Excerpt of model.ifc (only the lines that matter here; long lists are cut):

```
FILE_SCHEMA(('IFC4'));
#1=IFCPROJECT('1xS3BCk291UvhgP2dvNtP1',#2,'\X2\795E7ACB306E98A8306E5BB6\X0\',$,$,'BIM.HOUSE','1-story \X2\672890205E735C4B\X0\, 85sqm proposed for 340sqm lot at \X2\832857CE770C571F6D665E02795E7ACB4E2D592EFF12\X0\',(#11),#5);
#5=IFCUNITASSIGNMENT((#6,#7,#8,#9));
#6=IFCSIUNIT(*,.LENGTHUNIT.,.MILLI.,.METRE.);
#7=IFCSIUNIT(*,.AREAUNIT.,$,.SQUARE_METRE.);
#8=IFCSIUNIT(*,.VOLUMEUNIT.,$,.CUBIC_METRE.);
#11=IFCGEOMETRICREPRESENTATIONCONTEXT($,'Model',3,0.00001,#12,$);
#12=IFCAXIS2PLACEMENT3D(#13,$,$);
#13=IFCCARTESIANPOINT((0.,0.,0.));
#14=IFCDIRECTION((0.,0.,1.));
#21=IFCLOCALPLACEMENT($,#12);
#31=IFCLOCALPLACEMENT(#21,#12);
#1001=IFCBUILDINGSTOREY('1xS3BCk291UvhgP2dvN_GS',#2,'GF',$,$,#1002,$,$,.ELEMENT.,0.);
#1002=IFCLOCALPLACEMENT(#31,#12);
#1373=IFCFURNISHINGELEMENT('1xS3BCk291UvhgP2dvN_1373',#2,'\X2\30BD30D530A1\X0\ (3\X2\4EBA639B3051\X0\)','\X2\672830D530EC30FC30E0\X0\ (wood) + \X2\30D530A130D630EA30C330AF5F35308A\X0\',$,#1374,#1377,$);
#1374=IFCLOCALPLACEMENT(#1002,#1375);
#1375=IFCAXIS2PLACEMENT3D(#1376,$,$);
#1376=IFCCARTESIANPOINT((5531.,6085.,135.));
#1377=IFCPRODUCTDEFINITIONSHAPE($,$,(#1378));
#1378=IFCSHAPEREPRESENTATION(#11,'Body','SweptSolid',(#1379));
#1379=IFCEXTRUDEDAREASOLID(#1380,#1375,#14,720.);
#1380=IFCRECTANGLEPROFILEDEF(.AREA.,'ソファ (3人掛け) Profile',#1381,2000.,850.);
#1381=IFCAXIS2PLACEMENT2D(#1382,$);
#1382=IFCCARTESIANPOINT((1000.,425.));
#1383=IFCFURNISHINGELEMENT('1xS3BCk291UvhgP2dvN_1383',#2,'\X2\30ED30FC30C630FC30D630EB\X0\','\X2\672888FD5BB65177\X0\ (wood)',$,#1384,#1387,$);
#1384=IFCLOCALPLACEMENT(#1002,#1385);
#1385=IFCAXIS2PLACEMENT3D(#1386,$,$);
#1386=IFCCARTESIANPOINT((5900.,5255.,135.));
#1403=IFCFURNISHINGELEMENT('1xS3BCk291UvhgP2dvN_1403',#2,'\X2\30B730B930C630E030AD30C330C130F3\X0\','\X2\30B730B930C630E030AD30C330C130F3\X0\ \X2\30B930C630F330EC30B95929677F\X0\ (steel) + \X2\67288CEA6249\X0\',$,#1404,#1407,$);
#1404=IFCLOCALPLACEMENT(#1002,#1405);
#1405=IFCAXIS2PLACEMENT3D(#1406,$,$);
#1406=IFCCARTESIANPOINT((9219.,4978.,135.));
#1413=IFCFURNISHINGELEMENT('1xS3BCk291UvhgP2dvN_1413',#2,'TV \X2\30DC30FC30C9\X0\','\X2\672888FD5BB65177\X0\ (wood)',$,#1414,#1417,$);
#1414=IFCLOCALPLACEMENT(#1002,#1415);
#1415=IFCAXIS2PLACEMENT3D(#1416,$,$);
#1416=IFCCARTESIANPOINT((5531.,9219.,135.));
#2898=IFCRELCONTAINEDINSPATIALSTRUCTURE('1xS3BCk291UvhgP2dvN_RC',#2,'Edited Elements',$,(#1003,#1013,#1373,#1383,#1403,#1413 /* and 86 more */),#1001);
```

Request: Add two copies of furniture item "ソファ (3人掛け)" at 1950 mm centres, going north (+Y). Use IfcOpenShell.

```python
import numpy as np
import ifcopenshell
import ifcopenshell.api.geometry
import ifcopenshell.api.root
import ifcopenshell.util.element
import ifcopenshell.util.placement

model = ifcopenshell.open("model.ifc")


def reuse_history(source, copy):
    """copy_class also copies each property set's owner history, people and application; keep the originals."""
    for rel in copy.IsDefinedBy:
        if rel.is_a("IfcRelDefinesByProperties") and (history := rel.RelatingPropertyDefinition.OwnerHistory):
            rel.RelatingPropertyDefinition.OwnerHistory = source.OwnerHistory
            ifcopenshell.util.element.remove_deep2(model, history)


source = model.by_guid("1xS3BCk291UvhgP2dvN_1373")
base = ifcopenshell.util.placement.get_local_placement(source.ObjectPlacement)
step = np.array([0.0, 1.0, 0.0]) * 1950.0

for i in range(1, 3):
    copy = ifcopenshell.api.root.copy_class(model, product=source)
    copy.Representation = ifcopenshell.util.element.copy_deep(
        model, source.Representation, exclude=["IfcGeometricRepresentationContext", "IfcRepresentationMap"]
    )
    reuse_history(source, copy)
    matrix = base.copy()
    matrix[:3, 3] += i * step
    print("added at", matrix[:3, 3].round(3) + 0.0)
    ifcopenshell.api.geometry.edit_object_placement(model, product=copy, matrix=matrix, is_si=False)

model.write("model_v2.ifc")
```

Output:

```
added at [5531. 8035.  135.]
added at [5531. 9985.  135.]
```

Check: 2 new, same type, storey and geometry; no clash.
